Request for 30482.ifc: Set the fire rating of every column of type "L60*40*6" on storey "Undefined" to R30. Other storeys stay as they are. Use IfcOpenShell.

First a look at what the model holds.

```python
import ifcopenshell
import ifcopenshell.util.element

model = ifcopenshell.open("30482.ifc")
print(model.schema)
storey = next(s for s in model.by_type("IfcBuildingStorey") if s.Name == "Undefined")
columns = [e for e in ifcopenshell.util.element.get_decomposition(storey) if e.is_a("IfcColumn")]
seen = {}
for e in columns:
    element_type = ifcopenshell.util.element.get_type(e)
    key = (element_type.Name if element_type != e and element_type else None, ifcopenshell.util.element.get_pset(e, "Pset_ColumnCommon", "FireRating"))
    seen[key] = seen.get(key, 0) + 1
for (name, value), count in sorted(seen.items(), key=str):
    print(count, "x", name, "|", value)
```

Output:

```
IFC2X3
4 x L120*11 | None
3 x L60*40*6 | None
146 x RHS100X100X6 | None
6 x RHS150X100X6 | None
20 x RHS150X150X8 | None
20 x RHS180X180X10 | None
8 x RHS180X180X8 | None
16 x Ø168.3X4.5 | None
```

```python
import ifcopenshell
import ifcopenshell.api.pset
import ifcopenshell.util.element

model = ifcopenshell.open("30482.ifc")

storey = next(s for s in model.by_type("IfcBuildingStorey") if s.Name == "Undefined")
columns = [e for e in ifcopenshell.util.element.get_decomposition(storey) if e.is_a("IfcColumn")]

count = 0
for e in columns:
    element_type = ifcopenshell.util.element.get_type(e)
    if element_type in (None, e) or element_type.Name != "L60*40*6":
        continue
    # add_pset returns the element's existing set when there is one.
    pset = ifcopenshell.api.pset.add_pset(model, product=e, name="Pset_ColumnCommon")
    ifcopenshell.api.pset.edit_pset(model, pset=pset, properties={"FireRating": "R30"})
    count += 1

print(count, "columns updated")

model.write("30482_updated.ifc")
```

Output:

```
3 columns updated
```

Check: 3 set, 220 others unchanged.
